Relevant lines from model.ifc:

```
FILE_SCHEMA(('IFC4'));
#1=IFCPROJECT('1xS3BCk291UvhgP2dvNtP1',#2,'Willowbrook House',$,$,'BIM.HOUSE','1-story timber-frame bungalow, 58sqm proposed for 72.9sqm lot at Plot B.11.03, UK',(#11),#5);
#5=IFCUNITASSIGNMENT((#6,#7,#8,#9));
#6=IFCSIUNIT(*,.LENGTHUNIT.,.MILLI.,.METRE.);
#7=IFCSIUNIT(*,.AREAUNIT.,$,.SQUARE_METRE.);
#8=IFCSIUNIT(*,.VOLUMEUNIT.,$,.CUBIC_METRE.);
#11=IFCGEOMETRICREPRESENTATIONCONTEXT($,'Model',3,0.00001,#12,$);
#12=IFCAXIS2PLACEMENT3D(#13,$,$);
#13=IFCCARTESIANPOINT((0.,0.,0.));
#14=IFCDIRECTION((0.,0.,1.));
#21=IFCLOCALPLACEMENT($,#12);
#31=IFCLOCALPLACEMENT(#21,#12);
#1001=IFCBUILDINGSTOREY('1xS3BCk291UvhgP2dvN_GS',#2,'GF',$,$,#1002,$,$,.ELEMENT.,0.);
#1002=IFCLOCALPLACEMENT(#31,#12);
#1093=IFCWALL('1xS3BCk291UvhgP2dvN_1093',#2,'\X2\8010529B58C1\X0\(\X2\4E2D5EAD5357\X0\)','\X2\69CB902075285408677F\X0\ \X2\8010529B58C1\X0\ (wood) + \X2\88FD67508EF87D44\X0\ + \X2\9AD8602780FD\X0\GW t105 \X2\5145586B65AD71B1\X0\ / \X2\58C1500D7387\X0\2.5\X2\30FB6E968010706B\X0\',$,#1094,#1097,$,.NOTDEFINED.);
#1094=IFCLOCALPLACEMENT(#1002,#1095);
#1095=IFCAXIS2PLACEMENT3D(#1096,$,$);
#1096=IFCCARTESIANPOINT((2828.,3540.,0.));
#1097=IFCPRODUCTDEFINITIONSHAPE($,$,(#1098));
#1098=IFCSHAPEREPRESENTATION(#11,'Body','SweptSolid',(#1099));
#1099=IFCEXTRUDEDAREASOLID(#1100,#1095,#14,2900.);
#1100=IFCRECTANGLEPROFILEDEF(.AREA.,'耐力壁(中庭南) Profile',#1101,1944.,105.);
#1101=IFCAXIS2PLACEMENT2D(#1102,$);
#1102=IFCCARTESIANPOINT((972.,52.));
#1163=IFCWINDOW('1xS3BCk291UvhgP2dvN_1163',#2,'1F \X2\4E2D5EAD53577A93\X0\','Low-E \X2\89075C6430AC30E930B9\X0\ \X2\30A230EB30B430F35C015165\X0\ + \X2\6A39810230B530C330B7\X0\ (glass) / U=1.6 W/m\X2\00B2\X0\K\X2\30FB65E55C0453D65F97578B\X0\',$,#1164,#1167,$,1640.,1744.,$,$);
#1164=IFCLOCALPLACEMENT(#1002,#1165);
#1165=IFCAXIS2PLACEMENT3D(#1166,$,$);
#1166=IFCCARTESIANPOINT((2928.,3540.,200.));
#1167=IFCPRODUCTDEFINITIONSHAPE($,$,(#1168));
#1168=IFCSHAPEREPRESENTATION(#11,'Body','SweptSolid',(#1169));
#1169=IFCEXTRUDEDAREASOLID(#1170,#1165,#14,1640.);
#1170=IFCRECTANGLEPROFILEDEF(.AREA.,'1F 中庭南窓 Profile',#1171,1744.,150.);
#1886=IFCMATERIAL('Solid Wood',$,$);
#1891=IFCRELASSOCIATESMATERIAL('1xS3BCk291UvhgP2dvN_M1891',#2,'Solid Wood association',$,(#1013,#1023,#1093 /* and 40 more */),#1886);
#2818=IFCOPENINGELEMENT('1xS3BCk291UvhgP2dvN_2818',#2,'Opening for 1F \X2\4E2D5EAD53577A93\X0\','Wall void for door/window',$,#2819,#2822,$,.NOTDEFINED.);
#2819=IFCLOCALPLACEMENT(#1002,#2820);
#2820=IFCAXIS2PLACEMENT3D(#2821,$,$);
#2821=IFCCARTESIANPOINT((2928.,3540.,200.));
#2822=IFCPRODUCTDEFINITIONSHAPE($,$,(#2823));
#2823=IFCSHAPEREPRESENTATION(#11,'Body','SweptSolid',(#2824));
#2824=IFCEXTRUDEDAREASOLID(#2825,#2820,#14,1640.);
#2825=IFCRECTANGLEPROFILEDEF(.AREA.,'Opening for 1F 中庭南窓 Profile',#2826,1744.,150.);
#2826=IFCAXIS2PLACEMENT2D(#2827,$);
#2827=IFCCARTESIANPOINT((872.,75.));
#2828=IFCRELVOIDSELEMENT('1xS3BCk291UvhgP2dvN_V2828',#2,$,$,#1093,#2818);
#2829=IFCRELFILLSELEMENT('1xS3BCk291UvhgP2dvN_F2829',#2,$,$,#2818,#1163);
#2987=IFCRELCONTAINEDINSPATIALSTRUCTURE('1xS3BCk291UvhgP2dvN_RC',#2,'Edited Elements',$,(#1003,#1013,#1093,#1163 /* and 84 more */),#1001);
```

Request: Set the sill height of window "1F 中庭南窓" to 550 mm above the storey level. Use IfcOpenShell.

```python
import numpy as np
import ifcopenshell
import ifcopenshell.api.geometry
import ifcopenshell.geom
import ifcopenshell.util.element
import ifcopenshell.util.placement
import ifcopenshell.util.shape
import ifcopenshell.util.unit

model = ifcopenshell.open("model.ifc")
unit_scale = ifcopenshell.util.unit.calculate_unit_scale(model)

window = model.by_id(1163)
opening = window.FillsVoids[0].RelatingOpeningElement
storey = ifcopenshell.util.element.get_container(window, ifc_class="IfcBuildingStorey")
level = ifcopenshell.util.placement.get_local_placement(storey.ObjectPlacement)[2, 3]

# The opening's origin need not be at the sill, so measure its lowest point.
shape = ifcopenshell.geom.create_shape(ifcopenshell.geom.settings(), opening)
bottom = ifcopenshell.util.shape.get_shape_bottom_elevation(shape, shape.geometry) / unit_scale
dz = level + 0.55 / unit_scale - bottom

shift = np.array([0.0, 0.0, dz])
# The window is not placed relative to its opening, so move both.
for product in (opening, window):
    matrix = ifcopenshell.util.placement.get_local_placement(product.ObjectPlacement)
    matrix[:3, 3] += shift
    ifcopenshell.api.geometry.edit_object_placement(model, product=product, matrix=matrix, is_si=False)

print(f"moved by {dz * unit_scale:+.3f} m")

model.write("model_v2.ifc")
```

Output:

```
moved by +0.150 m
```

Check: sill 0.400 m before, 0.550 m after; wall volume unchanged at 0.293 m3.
